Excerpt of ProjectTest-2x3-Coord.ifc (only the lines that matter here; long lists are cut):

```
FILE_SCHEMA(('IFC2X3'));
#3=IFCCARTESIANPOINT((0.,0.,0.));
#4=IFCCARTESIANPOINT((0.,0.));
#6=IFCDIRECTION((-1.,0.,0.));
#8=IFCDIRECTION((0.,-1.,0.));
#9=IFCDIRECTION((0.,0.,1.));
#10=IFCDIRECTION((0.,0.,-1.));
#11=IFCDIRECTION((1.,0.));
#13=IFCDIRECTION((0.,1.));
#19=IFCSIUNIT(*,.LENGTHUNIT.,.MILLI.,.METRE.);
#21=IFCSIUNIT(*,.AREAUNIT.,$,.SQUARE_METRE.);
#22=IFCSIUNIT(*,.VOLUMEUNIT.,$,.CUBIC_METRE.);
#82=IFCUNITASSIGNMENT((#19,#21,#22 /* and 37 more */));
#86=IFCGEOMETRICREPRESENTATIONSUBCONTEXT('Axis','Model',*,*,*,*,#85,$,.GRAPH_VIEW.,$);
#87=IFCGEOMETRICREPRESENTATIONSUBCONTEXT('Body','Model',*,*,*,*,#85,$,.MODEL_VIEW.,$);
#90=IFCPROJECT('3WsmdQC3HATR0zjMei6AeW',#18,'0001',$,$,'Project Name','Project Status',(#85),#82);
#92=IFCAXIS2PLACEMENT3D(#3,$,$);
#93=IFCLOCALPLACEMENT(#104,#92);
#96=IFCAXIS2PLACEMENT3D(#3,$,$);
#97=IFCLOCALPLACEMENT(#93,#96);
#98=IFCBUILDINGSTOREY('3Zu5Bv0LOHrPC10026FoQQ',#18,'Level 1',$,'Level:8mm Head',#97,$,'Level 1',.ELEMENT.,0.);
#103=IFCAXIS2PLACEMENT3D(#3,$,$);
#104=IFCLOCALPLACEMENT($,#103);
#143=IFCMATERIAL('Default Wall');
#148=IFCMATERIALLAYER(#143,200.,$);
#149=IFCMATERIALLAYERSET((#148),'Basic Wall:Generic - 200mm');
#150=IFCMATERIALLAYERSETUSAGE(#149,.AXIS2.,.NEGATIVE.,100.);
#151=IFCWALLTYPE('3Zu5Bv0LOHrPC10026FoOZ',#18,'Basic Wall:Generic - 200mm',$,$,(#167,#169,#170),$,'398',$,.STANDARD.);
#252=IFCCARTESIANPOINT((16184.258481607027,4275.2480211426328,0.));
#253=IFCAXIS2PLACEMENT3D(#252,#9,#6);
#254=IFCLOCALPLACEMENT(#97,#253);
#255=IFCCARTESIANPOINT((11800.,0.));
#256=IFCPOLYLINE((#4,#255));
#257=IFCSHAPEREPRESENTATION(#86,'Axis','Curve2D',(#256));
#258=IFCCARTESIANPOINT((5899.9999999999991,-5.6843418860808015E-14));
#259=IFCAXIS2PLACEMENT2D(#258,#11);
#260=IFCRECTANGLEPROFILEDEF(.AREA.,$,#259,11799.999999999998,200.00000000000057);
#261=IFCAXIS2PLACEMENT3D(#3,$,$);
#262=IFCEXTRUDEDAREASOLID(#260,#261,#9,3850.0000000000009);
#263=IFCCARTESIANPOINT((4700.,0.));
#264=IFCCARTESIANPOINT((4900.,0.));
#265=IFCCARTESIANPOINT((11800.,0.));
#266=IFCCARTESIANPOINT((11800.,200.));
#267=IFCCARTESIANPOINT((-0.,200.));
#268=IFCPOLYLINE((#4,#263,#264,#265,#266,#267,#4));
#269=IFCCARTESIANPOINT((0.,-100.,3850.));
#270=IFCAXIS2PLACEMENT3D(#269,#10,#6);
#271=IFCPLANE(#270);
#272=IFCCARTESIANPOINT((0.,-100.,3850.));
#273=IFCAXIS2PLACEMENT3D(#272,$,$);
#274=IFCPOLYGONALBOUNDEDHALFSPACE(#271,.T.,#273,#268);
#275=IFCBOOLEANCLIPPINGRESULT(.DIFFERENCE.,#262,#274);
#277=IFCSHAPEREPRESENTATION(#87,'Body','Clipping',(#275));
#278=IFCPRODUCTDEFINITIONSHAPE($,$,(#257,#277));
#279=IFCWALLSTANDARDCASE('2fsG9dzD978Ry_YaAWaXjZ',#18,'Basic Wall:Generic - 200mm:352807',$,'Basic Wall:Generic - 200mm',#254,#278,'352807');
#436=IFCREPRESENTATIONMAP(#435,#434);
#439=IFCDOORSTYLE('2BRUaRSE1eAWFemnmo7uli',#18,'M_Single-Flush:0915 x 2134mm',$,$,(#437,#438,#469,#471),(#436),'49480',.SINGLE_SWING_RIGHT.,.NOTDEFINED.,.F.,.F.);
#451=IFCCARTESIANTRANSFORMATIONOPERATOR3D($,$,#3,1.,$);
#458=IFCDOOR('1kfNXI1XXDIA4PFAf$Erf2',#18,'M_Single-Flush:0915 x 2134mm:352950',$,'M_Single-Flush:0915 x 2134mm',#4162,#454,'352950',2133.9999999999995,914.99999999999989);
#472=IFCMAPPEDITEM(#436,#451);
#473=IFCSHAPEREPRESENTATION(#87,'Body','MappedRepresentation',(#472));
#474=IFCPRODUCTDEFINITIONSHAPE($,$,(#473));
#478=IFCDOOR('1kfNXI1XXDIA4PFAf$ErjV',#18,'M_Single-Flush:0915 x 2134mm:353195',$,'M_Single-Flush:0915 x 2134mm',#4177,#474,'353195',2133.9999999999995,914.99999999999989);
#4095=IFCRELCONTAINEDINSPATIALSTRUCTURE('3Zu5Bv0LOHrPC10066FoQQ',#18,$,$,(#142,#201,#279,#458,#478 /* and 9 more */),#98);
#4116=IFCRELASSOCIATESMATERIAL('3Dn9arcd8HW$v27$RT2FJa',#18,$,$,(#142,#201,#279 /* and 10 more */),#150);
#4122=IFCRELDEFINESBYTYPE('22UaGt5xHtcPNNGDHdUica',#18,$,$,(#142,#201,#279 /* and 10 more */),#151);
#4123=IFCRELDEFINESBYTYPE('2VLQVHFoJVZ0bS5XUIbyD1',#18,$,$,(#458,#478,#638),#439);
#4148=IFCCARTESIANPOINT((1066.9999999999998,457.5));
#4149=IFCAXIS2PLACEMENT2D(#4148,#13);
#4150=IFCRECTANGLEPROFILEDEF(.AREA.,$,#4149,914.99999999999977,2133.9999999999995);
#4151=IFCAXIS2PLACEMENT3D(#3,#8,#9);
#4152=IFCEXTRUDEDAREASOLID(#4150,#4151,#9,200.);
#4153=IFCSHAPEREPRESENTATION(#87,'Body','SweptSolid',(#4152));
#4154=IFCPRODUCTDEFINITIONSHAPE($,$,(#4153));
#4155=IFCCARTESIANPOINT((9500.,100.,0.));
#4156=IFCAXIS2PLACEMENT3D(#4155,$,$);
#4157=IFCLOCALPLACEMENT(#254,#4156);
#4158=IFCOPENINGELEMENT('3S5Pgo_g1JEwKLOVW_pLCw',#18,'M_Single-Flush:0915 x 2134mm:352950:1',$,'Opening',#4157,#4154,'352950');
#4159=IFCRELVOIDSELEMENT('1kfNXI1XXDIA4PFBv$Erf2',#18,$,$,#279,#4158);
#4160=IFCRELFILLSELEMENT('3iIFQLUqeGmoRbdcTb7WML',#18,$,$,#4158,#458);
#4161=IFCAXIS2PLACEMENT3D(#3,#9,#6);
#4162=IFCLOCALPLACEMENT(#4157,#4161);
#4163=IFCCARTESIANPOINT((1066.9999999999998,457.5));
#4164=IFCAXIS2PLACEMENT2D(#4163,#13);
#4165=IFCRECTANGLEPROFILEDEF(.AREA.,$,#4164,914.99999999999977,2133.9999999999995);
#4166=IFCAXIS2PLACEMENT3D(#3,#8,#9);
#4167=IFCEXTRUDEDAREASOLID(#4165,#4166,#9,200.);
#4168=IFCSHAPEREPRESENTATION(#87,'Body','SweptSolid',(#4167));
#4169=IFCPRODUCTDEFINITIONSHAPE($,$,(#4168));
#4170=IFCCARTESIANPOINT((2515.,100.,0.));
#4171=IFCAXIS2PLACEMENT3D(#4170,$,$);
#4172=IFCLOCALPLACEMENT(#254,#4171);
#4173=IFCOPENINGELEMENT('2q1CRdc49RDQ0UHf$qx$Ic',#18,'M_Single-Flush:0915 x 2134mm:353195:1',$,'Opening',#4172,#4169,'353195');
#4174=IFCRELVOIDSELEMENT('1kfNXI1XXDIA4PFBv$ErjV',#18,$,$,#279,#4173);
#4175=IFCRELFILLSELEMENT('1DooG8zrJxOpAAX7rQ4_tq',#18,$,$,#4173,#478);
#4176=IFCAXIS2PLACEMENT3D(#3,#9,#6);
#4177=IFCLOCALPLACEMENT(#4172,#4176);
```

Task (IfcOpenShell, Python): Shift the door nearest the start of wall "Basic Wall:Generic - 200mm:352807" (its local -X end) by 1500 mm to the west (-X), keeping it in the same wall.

```python
import ifcopenshell
import ifcopenshell.api.geometry
import ifcopenshell.util.placement

model = ifcopenshell.open("ProjectTest-2x3-Coord.ifc")

door = model.by_guid("1kfNXI1XXDIA4PFAf$ErjV")
opening = door.FillsVoids[0].RelatingOpeningElement
wall = opening.VoidsElements[0].RelatingBuildingElement

wall_matrix = ifcopenshell.util.placement.get_local_placement(wall.ObjectPlacement)
shift = wall_matrix[:3, 0] * 1500.0
before = ifcopenshell.util.placement.get_local_placement(door.ObjectPlacement)[:3, 3].copy()

# The door is placed relative to its opening, so it follows when the opening moves.
matrix = ifcopenshell.util.placement.get_local_placement(opening.ObjectPlacement)
matrix[:3, 3] += shift
ifcopenshell.api.geometry.edit_object_placement(
    model, product=opening, matrix=matrix, is_si=False, should_transform_children=True
)

after = ifcopenshell.util.placement.get_local_placement(door.ObjectPlacement)[:3, 3]
print("door moved by", (after - before).round(3) + 0.0)

model.write("ProjectTest-2x3-Coord_edited.ifc")
```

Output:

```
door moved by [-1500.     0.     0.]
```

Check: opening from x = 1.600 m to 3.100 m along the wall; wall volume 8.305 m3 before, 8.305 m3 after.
